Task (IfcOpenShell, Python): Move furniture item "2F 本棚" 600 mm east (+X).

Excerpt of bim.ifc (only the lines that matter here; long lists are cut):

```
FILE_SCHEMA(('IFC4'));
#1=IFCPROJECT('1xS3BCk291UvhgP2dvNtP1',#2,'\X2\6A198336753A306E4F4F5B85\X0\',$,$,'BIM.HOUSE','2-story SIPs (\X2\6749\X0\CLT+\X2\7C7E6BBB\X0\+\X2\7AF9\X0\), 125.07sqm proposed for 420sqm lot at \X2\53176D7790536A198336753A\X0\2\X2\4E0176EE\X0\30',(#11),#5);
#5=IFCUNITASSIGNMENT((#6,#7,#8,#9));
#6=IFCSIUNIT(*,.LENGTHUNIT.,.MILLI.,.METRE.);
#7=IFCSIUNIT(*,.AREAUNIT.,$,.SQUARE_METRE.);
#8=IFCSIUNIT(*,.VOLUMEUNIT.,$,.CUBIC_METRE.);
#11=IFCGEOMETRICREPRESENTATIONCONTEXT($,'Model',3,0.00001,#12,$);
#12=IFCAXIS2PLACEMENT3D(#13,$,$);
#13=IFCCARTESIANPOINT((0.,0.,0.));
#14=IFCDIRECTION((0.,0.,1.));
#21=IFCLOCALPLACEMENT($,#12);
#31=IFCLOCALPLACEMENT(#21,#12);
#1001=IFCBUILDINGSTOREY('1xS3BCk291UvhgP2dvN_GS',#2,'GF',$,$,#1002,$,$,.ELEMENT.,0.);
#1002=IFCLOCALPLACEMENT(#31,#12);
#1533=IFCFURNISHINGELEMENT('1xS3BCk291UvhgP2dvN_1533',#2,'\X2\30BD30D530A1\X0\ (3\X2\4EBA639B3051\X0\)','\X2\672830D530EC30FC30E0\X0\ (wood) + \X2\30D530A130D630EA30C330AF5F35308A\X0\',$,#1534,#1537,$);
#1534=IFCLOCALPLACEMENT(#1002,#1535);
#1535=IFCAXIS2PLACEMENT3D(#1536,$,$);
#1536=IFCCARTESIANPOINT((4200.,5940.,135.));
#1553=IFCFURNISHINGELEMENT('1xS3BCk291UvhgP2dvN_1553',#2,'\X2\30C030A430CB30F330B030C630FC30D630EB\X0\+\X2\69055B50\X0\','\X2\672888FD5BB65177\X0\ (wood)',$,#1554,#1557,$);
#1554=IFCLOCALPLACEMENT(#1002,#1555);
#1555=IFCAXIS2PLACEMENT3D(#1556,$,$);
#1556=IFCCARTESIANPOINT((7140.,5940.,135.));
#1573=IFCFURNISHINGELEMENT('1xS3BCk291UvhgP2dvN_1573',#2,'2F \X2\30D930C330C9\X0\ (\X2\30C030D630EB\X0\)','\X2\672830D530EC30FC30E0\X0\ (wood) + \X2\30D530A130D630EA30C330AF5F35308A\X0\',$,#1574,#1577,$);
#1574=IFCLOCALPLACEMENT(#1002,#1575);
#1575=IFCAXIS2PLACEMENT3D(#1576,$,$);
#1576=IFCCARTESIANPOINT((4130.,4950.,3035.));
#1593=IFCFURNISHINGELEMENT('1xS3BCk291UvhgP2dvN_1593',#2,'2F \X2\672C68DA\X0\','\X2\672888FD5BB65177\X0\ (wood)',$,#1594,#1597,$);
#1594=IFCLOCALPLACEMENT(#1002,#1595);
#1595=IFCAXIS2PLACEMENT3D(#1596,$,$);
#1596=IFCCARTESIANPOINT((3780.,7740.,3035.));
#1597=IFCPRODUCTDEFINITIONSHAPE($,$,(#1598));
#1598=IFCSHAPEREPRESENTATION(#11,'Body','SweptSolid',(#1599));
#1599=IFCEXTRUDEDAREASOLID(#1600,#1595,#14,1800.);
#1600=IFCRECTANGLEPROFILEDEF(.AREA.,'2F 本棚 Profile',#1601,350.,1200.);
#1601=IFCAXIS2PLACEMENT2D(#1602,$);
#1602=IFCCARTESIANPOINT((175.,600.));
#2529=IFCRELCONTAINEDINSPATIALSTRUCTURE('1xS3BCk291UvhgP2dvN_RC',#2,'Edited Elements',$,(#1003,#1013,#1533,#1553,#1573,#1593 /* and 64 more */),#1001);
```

```python
import ifcopenshell
import ifcopenshell.api.geometry
import ifcopenshell.util.placement
import ifcopenshell.util.unit

model = ifcopenshell.open("bim.ifc")
unit_scale = ifcopenshell.util.unit.calculate_unit_scale(model)

item = model.by_guid("1xS3BCk291UvhgP2dvN_1593")
matrix = ifcopenshell.util.placement.get_local_placement(item.ObjectPlacement)
matrix[0, 3] += 0.6 / unit_scale
ifcopenshell.api.geometry.edit_object_placement(model, product=item, matrix=matrix, is_si=False)

print(ifcopenshell.util.placement.get_local_placement(item.ObjectPlacement).round(3) + 0.0)

model.write("bim_edited.ifc")
```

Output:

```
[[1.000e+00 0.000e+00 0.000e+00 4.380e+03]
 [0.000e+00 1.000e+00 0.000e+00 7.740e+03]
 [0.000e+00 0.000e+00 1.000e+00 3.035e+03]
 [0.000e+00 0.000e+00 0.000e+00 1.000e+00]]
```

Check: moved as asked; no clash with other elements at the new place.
